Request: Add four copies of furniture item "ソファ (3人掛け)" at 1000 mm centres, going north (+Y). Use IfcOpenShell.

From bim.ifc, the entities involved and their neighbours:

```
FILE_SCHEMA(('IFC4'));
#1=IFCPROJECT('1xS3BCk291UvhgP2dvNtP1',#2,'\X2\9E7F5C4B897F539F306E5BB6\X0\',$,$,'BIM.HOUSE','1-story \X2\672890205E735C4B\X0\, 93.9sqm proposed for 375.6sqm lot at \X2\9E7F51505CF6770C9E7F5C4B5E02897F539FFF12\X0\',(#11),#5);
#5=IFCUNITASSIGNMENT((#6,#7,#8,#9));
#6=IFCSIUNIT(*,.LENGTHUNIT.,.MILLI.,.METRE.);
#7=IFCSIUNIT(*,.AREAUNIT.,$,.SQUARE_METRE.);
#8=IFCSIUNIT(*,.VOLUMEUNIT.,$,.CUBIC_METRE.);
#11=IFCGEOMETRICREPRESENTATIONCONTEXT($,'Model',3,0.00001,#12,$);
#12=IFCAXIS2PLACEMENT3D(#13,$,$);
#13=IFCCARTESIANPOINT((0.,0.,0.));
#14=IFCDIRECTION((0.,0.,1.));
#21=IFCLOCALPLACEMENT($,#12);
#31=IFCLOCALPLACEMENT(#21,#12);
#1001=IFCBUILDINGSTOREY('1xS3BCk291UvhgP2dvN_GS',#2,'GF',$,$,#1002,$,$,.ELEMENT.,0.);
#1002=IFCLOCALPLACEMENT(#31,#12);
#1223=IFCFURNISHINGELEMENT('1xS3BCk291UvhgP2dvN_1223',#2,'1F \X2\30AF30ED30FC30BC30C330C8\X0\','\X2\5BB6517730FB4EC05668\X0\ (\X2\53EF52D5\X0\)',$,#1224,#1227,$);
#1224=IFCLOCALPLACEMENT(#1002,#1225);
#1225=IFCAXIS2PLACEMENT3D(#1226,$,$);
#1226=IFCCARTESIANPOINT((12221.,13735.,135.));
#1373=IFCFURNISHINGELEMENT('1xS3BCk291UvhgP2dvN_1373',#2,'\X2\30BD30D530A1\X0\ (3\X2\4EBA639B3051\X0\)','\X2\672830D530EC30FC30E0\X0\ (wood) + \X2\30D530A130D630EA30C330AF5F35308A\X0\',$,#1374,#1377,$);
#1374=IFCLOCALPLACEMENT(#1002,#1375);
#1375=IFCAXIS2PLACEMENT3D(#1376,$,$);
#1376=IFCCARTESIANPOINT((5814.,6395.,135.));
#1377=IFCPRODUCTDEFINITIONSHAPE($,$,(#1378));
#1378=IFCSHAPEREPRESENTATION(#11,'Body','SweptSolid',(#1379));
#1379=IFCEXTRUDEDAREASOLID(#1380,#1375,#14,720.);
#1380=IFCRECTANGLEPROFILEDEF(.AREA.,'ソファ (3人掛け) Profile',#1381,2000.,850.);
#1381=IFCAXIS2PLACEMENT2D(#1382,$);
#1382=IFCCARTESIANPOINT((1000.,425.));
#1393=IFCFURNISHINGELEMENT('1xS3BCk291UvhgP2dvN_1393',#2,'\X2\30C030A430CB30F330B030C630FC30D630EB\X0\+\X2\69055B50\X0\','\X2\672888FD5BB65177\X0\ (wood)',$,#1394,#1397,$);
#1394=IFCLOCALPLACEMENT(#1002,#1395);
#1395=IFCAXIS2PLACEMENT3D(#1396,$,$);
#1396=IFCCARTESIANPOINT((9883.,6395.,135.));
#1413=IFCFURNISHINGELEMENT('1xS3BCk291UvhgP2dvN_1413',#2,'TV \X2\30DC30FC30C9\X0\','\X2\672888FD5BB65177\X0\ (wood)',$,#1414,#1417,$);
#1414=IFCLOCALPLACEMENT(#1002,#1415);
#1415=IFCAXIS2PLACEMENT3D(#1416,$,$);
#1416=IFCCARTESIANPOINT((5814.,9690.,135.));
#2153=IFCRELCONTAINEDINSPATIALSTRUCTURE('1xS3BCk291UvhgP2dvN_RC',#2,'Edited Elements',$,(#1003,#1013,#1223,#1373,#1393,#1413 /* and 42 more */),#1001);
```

```python
import numpy as np
import ifcopenshell
import ifcopenshell.api.geometry
import ifcopenshell.api.root
import ifcopenshell.util.element
import ifcopenshell.util.placement
import ifcopenshell.util.unit

model = ifcopenshell.open("bim.ifc")
unit_scale = ifcopenshell.util.unit.calculate_unit_scale(model)


def reuse_history(source, copy):
    """copy_class also copies each property set's owner history, people and application; keep the originals."""
    for rel in copy.IsDefinedBy:
        if rel.is_a("IfcRelDefinesByProperties") and (history := rel.RelatingPropertyDefinition.OwnerHistory):
            rel.RelatingPropertyDefinition.OwnerHistory = source.OwnerHistory
            ifcopenshell.util.element.remove_deep2(model, history)


source = model.by_id(1373)
base = ifcopenshell.util.placement.get_local_placement(source.ObjectPlacement)
step = np.array([0.0, 1.0, 0.0]) * 1 / unit_scale

for i in range(1, 5):
    copy = ifcopenshell.api.root.copy_class(model, product=source)
    copy.Representation = ifcopenshell.util.element.copy_deep(
        model, source.Representation, exclude=["IfcGeometricRepresentationContext", "IfcRepresentationMap"]
    )
    reuse_history(source, copy)
    matrix = base.copy()
    matrix[:3, 3] += i * step
    print("added at", matrix[:3, 3].round(3) + 0.0)
    ifcopenshell.api.geometry.edit_object_placement(model, product=copy, matrix=matrix, is_si=False)

model.write("bim_rev.ifc")
```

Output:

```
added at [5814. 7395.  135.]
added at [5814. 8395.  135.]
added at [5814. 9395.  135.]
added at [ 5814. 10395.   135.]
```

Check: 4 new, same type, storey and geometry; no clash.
